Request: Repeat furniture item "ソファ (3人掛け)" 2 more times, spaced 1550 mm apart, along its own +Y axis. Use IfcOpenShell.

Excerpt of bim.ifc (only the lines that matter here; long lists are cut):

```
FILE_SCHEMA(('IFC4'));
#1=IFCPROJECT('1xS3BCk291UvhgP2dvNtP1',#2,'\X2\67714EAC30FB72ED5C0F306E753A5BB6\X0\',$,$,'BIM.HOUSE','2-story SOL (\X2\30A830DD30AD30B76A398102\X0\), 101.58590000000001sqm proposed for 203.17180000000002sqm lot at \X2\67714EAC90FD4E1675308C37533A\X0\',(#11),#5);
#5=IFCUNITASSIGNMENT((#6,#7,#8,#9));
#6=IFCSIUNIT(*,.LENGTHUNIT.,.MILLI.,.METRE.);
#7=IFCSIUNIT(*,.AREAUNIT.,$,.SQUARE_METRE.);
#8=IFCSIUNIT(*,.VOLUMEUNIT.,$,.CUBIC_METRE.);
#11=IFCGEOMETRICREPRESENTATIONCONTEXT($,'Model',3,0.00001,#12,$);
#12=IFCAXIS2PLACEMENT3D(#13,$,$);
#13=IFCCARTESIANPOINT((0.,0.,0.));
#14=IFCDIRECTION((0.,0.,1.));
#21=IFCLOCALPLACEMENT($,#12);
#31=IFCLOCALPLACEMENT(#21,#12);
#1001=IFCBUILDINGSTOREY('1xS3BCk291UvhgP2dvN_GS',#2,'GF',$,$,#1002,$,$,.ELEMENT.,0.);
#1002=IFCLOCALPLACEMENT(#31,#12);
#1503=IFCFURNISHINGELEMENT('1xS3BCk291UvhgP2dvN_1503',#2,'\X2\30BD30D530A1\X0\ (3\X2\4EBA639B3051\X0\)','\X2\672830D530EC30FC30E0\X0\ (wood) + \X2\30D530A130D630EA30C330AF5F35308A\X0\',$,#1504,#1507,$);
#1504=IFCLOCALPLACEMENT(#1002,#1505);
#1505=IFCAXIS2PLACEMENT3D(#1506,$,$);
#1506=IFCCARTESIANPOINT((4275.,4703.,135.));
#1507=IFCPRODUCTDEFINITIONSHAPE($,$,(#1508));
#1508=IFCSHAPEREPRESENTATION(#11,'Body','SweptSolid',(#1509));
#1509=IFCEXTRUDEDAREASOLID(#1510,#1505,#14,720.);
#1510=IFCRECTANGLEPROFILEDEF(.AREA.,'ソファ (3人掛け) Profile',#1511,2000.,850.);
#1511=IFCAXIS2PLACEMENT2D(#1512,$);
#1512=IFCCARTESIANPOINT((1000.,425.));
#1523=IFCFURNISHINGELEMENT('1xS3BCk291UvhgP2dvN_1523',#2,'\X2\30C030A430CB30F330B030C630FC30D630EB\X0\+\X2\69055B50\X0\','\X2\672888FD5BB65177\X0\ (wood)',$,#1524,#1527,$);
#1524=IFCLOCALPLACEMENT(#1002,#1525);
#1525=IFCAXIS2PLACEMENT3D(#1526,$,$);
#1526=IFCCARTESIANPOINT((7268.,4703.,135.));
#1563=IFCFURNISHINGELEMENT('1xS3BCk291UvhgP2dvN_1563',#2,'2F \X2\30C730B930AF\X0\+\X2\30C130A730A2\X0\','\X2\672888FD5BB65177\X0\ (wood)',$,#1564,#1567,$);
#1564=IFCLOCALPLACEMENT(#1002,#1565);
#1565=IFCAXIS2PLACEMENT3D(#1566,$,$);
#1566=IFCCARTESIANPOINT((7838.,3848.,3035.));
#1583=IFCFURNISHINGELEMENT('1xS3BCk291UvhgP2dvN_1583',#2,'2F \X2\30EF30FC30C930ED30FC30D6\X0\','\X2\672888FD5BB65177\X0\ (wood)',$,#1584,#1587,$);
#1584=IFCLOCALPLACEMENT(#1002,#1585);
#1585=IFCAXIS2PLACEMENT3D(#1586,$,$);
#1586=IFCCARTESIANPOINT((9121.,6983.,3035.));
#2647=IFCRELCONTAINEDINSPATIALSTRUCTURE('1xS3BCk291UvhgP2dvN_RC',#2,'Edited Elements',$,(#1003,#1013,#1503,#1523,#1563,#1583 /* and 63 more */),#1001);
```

```python
import ifcopenshell
import ifcopenshell.api.geometry
import ifcopenshell.api.root
import ifcopenshell.util.element
import ifcopenshell.util.placement
import ifcopenshell.util.unit

model = ifcopenshell.open("bim.ifc")
unit_scale = ifcopenshell.util.unit.calculate_unit_scale(model)


def reuse_history(source, copy):
    """copy_class also copies each property set's owner history, people and application; keep the originals."""
    for rel in copy.IsDefinedBy:
        if rel.is_a("IfcRelDefinesByProperties") and (history := rel.RelatingPropertyDefinition.OwnerHistory):
            rel.RelatingPropertyDefinition.OwnerHistory = source.OwnerHistory
            ifcopenshell.util.element.remove_deep2(model, history)


source = model.by_guid("1xS3BCk291UvhgP2dvN_1503")
base = ifcopenshell.util.placement.get_local_placement(source.ObjectPlacement)
step = base[:3, 1] * 1.55 / unit_scale

for i in range(1, 3):
    copy = ifcopenshell.api.root.copy_class(model, product=source)
    copy.Representation = ifcopenshell.util.element.copy_deep(
        model, source.Representation, exclude=["IfcGeometricRepresentationContext", "IfcRepresentationMap"]
    )
    reuse_history(source, copy)
    matrix = base.copy()
    matrix[:3, 3] += i * step
    print("added at", matrix[:3, 3].round(3) + 0.0)
    ifcopenshell.api.geometry.edit_object_placement(model, product=copy, matrix=matrix, is_si=False)

model.write("bim_updated.ifc")
```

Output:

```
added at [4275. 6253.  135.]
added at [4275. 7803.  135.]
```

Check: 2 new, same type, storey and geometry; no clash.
